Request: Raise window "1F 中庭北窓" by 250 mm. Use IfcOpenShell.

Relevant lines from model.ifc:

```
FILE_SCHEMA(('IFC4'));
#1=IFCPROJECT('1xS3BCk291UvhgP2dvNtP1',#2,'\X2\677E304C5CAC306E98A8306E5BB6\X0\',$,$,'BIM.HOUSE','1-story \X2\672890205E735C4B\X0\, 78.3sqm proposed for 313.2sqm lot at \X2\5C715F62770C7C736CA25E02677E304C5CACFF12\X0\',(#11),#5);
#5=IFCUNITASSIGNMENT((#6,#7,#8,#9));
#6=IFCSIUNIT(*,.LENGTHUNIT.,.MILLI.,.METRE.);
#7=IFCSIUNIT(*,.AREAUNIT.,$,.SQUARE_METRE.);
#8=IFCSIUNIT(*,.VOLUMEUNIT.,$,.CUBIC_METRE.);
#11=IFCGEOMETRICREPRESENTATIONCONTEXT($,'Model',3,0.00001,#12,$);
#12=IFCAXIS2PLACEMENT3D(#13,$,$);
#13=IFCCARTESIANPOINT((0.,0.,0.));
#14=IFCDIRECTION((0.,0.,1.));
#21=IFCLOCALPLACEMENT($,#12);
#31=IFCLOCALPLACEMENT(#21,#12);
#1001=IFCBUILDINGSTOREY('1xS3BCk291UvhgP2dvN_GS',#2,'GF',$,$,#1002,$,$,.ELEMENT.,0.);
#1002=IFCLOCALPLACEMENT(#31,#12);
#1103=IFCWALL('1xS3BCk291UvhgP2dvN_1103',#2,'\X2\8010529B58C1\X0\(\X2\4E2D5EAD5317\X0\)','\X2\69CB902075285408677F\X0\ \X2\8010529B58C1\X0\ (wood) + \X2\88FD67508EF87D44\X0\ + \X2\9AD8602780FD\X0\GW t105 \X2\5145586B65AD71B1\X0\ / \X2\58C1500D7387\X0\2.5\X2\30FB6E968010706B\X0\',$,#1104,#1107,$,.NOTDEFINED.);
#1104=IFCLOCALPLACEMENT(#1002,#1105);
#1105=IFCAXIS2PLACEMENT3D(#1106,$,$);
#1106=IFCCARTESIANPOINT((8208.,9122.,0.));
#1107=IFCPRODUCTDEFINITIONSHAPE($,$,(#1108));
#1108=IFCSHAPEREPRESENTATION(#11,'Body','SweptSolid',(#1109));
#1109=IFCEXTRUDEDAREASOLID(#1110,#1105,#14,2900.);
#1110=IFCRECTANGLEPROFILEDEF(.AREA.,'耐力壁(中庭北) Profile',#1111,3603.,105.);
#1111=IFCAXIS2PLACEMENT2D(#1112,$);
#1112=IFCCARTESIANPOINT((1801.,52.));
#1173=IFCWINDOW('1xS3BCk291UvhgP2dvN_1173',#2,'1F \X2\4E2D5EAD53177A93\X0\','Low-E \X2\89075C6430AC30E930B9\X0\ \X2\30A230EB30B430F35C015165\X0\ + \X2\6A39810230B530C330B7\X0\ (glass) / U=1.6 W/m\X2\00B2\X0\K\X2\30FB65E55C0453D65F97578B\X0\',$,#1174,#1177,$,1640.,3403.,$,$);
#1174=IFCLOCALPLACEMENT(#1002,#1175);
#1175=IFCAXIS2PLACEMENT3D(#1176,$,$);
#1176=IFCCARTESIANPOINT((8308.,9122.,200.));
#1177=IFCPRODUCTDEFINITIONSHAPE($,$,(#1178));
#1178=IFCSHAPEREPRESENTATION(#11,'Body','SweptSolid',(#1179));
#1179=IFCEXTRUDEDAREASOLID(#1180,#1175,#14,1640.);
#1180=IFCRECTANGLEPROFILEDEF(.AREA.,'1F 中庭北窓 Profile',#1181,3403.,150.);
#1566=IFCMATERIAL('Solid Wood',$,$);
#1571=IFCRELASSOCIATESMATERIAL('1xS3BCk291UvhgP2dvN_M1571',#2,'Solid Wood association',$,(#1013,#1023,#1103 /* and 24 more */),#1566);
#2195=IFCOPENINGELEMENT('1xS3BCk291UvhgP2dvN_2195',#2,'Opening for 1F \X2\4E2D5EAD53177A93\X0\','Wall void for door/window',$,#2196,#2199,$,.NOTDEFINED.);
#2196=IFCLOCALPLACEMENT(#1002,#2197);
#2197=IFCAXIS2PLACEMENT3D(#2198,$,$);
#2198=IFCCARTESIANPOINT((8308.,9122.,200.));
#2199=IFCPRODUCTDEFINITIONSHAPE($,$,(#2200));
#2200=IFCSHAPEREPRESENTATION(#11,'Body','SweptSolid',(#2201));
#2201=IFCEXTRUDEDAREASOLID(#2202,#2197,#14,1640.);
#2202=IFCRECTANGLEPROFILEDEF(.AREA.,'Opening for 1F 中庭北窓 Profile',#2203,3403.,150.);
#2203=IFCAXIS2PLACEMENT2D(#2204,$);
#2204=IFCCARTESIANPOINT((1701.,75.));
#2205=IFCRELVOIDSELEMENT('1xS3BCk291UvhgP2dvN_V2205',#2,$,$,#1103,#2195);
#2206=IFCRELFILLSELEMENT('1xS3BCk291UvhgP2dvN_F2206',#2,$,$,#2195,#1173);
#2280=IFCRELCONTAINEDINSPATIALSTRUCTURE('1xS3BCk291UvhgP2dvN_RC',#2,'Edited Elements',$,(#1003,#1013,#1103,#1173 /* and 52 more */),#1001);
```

```python
import numpy as np
import ifcopenshell
import ifcopenshell.api.geometry
import ifcopenshell.util.placement
import ifcopenshell.util.unit

model = ifcopenshell.open("model.ifc")
unit_scale = ifcopenshell.util.unit.calculate_unit_scale(model)

window = model.by_guid("1xS3BCk291UvhgP2dvN_1173")
opening = window.FillsVoids[0].RelatingOpeningElement
dz = 0.25 / unit_scale

shift = np.array([0.0, 0.0, dz])
# The window is not placed relative to its opening, so move both.
for product in (opening, window):
    matrix = ifcopenshell.util.placement.get_local_placement(product.ObjectPlacement)
    matrix[:3, 3] += shift
    ifcopenshell.api.geometry.edit_object_placement(model, product=product, matrix=matrix, is_si=False)

print(f"moved by {dz * unit_scale:+.3f} m")

model.write("model_rev.ifc")
```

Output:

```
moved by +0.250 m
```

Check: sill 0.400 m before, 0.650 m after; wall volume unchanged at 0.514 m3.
